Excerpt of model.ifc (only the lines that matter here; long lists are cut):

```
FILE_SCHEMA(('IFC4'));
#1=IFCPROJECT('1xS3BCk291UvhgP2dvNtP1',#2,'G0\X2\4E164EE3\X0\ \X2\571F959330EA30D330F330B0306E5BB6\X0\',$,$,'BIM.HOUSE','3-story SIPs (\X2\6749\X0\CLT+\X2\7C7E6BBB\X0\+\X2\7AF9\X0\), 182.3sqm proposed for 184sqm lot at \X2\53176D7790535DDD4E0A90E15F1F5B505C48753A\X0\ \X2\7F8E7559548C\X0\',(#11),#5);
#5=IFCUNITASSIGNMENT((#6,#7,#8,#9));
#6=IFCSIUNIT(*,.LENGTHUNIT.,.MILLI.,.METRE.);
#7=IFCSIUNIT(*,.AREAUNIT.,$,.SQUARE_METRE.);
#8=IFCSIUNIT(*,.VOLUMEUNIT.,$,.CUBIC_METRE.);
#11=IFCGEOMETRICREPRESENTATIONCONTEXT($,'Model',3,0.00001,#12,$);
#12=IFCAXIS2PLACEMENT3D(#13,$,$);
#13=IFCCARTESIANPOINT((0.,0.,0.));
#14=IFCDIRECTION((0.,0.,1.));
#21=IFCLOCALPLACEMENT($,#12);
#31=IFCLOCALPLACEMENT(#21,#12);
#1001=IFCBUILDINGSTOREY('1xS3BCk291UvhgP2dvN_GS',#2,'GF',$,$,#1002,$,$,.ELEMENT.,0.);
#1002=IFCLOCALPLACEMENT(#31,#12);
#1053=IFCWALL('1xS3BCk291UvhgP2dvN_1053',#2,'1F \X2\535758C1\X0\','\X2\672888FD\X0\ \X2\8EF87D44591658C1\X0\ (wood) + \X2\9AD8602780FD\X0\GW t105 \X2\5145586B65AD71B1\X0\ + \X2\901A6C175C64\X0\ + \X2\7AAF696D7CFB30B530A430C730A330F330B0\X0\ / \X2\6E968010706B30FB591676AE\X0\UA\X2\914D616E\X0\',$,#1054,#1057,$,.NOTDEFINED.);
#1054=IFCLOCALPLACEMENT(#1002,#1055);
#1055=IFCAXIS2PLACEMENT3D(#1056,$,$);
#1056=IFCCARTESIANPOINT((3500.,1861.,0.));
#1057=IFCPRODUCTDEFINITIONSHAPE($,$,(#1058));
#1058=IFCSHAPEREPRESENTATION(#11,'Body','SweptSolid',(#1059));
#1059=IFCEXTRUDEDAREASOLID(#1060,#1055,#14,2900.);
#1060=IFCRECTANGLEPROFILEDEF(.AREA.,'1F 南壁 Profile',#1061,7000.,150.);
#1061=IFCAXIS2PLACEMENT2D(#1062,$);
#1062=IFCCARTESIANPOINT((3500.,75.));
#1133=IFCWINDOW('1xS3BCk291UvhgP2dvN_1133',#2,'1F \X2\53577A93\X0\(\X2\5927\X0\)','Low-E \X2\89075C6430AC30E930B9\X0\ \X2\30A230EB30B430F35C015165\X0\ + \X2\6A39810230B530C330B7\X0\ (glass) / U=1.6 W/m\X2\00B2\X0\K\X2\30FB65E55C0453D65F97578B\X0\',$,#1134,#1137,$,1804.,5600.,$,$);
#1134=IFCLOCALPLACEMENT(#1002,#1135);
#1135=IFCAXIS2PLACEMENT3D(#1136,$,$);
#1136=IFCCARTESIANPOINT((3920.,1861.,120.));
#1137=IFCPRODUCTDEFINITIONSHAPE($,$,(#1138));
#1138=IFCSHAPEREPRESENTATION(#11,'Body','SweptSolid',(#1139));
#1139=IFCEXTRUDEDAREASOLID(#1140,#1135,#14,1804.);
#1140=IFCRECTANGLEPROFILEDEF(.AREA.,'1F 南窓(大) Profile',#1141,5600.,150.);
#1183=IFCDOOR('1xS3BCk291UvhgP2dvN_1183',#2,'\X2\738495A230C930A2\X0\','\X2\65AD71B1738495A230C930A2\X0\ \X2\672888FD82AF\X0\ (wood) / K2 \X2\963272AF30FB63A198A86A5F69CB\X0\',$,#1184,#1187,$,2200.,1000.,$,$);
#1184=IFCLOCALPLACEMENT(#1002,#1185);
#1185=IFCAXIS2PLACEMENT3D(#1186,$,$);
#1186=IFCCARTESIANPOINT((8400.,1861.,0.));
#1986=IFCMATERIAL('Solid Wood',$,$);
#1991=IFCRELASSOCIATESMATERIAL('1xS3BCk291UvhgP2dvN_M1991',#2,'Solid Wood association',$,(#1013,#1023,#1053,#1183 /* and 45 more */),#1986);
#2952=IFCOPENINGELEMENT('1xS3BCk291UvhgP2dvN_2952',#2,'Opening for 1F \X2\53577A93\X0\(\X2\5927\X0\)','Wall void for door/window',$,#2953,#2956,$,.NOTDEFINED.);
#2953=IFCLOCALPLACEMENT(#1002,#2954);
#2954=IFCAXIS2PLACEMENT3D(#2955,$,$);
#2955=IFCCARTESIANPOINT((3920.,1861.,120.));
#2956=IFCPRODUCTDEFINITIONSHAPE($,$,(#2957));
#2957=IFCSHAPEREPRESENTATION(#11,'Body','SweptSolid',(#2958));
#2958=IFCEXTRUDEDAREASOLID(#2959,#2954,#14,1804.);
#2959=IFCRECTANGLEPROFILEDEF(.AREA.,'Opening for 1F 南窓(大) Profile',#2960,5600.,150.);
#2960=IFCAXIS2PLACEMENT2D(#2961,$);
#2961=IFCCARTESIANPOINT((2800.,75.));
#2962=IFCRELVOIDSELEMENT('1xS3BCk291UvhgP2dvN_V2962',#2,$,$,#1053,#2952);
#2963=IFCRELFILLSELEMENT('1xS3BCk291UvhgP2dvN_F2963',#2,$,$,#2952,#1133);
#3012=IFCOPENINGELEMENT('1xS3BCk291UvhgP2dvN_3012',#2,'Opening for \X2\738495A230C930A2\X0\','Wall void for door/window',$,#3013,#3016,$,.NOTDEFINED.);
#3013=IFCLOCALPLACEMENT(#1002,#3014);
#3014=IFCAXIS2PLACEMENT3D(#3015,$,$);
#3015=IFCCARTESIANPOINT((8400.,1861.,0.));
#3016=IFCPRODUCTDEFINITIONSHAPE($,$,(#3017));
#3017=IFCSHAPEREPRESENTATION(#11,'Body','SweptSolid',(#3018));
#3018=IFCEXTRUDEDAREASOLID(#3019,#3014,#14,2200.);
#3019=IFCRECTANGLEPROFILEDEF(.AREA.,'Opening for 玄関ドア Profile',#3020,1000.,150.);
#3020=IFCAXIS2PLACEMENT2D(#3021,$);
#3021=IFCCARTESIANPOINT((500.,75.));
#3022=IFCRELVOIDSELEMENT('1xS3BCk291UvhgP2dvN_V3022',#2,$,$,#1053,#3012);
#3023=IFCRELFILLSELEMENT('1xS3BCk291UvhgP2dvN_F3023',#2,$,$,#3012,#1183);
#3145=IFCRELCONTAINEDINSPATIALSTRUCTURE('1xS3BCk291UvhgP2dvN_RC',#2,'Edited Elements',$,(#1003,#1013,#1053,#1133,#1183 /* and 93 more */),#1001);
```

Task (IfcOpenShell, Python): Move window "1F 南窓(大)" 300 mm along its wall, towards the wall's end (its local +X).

```python
import ifcopenshell
import ifcopenshell.api.geometry
import ifcopenshell.util.placement

model = ifcopenshell.open("model.ifc")

window = model.by_id(1133)
opening = window.FillsVoids[0].RelatingOpeningElement
wall = opening.VoidsElements[0].RelatingBuildingElement

wall_matrix = ifcopenshell.util.placement.get_local_placement(wall.ObjectPlacement)
shift = wall_matrix[:3, 0] * 300.0
before = ifcopenshell.util.placement.get_local_placement(window.ObjectPlacement)[:3, 3].copy()

# The window is not placed relative to its opening, so move both.
for product in (opening, window):
    matrix = ifcopenshell.util.placement.get_local_placement(product.ObjectPlacement)
    matrix[:3, 3] += shift
    ifcopenshell.api.geometry.edit_object_placement(model, product=product, matrix=matrix, is_si=False)

after = ifcopenshell.util.placement.get_local_placement(window.ObjectPlacement)[:3, 3]
print("window moved by", (after - before).round(3) + 0.0)

model.write("model-out.ifc")
```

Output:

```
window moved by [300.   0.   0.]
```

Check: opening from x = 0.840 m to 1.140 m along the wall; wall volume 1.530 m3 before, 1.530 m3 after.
